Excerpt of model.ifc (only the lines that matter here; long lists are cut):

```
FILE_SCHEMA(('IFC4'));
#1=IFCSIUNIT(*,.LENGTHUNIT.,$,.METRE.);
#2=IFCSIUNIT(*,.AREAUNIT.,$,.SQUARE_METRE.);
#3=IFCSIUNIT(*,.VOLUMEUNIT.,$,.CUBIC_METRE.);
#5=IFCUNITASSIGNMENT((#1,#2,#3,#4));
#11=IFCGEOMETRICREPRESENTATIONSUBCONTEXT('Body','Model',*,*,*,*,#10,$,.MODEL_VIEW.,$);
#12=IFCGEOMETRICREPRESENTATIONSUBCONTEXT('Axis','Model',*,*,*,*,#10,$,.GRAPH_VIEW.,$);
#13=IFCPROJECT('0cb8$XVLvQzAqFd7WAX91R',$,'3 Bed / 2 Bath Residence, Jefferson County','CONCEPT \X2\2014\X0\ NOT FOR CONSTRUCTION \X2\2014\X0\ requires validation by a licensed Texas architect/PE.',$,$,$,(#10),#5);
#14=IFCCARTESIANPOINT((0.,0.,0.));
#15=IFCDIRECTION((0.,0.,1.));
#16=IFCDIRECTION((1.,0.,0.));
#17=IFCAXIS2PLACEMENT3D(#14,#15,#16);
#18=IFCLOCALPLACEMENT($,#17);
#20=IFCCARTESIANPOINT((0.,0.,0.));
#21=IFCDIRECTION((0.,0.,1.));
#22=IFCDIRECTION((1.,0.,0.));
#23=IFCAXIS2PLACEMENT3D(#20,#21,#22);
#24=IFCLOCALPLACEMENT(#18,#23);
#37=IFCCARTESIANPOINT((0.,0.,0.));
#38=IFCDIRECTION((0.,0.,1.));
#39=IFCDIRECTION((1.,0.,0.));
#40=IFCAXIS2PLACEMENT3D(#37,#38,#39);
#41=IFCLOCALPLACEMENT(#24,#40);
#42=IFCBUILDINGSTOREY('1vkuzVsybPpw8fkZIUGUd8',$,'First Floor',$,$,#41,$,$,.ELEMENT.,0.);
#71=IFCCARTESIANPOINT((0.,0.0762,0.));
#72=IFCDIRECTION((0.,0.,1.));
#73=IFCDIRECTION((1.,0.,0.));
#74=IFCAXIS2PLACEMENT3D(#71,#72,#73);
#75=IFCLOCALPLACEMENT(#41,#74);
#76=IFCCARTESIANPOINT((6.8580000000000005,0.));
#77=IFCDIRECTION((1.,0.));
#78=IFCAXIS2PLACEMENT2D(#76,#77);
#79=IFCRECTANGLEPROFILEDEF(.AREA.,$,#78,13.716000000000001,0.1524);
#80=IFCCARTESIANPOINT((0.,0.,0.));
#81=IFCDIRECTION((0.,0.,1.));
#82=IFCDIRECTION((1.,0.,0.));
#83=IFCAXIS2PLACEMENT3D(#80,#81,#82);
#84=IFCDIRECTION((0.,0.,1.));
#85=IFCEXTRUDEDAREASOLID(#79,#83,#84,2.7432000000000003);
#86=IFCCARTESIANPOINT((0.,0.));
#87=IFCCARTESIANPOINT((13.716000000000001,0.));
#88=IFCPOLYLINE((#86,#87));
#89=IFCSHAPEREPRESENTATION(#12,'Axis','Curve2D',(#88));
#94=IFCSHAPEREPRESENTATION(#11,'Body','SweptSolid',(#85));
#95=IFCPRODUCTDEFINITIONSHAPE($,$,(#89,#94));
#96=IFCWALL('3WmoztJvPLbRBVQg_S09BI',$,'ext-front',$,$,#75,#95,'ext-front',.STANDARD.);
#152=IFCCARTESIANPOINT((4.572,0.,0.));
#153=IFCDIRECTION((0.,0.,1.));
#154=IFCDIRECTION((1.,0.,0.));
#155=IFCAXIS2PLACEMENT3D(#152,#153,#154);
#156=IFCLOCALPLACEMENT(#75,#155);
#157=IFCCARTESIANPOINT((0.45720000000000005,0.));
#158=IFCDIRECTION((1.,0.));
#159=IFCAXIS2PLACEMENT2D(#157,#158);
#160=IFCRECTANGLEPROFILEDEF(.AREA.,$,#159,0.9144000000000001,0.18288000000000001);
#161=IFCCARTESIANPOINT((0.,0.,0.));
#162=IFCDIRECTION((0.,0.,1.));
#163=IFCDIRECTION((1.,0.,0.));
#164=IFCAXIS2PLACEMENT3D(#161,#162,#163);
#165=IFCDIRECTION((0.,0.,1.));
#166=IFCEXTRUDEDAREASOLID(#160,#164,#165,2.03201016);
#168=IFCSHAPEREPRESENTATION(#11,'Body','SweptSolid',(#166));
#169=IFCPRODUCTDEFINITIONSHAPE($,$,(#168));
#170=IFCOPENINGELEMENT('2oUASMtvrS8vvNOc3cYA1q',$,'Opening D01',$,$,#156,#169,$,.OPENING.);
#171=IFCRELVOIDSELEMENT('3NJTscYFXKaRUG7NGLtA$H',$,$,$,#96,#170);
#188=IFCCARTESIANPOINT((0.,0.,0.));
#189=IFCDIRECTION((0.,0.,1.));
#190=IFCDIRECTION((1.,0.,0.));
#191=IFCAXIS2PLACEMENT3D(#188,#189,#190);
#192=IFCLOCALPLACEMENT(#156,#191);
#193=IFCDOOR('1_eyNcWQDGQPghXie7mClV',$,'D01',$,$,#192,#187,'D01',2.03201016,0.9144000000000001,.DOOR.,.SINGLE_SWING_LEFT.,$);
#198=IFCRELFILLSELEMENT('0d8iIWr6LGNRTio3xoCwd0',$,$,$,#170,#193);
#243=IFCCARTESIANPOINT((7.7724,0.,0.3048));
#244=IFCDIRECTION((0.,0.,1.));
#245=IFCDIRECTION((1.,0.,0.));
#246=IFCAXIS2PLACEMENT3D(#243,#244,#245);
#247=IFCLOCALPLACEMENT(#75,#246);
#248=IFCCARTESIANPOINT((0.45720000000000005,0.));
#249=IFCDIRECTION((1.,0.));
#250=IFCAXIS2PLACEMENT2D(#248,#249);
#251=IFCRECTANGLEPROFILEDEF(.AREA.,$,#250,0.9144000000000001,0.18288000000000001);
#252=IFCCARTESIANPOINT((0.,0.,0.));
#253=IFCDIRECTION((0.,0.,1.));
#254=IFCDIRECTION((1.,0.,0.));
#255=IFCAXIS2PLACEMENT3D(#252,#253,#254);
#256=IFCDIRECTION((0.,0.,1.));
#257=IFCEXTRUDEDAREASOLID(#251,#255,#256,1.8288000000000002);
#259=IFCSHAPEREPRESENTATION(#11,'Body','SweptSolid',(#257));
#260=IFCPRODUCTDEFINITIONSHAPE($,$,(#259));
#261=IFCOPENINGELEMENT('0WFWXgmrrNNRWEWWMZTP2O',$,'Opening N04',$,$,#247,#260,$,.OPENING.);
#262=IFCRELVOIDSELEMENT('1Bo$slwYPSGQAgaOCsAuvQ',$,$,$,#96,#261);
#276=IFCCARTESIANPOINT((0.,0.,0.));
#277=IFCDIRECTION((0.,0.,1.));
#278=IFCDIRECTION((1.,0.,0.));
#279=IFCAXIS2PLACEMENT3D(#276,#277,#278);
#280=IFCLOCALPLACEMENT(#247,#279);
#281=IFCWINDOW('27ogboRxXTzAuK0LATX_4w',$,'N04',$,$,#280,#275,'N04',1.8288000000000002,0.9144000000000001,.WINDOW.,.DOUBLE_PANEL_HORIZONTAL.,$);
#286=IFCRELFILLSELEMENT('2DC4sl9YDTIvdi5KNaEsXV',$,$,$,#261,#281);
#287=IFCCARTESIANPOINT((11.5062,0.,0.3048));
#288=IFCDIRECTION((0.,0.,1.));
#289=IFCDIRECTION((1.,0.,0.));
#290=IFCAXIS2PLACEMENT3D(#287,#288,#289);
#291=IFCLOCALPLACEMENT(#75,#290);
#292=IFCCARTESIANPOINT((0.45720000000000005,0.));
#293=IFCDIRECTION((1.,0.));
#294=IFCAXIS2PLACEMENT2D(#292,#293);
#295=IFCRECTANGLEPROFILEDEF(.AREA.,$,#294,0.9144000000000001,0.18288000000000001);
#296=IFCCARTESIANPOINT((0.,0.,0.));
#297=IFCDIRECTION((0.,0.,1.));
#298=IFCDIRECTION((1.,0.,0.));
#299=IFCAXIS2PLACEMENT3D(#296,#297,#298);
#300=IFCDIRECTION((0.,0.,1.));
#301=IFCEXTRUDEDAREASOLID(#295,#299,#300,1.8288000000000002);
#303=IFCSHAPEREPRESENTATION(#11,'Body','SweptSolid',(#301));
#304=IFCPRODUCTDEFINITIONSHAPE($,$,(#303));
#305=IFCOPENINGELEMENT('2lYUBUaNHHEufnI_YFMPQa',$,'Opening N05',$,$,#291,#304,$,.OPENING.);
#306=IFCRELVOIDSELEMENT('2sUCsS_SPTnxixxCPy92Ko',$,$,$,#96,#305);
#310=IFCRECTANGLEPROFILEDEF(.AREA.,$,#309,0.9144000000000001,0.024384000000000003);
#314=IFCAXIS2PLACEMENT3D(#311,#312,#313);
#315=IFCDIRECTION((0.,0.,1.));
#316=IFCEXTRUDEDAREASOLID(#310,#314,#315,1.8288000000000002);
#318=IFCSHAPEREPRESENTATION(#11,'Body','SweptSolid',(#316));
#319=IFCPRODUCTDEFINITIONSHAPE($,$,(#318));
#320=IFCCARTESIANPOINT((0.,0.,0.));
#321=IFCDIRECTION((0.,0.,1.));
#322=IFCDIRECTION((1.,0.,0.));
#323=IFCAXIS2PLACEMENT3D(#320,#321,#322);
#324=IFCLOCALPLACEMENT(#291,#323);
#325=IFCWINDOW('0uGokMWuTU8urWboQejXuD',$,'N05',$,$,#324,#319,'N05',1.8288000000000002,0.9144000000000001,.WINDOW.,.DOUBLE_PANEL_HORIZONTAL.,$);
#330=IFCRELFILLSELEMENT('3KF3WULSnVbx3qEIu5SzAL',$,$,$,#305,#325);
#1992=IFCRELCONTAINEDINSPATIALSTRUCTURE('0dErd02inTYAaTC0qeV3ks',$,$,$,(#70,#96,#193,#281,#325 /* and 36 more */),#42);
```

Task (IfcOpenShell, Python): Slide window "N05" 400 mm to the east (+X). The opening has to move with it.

```python
import ifcopenshell
import ifcopenshell.api.geometry
import ifcopenshell.util.placement

model = ifcopenshell.open("model.ifc")

window = model.by_id(325)
opening = window.FillsVoids[0].RelatingOpeningElement
wall = opening.VoidsElements[0].RelatingBuildingElement

wall_matrix = ifcopenshell.util.placement.get_local_placement(wall.ObjectPlacement)
shift = wall_matrix[:3, 0] * 0.4
before = ifcopenshell.util.placement.get_local_placement(window.ObjectPlacement)[:3, 3].copy()

# The window is placed relative to its opening, so it follows when the opening moves.
matrix = ifcopenshell.util.placement.get_local_placement(opening.ObjectPlacement)
matrix[:3, 3] += shift
ifcopenshell.api.geometry.edit_object_placement(
    model, product=opening, matrix=matrix, is_si=False, should_transform_children=True
)

after = ifcopenshell.util.placement.get_local_placement(window.ObjectPlacement)[:3, 3]
print("window moved by", (after - before).round(3) + 0.0)

model.write("model_rev.ifc")
```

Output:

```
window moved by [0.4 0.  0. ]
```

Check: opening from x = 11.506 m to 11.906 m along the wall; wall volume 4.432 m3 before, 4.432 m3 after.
